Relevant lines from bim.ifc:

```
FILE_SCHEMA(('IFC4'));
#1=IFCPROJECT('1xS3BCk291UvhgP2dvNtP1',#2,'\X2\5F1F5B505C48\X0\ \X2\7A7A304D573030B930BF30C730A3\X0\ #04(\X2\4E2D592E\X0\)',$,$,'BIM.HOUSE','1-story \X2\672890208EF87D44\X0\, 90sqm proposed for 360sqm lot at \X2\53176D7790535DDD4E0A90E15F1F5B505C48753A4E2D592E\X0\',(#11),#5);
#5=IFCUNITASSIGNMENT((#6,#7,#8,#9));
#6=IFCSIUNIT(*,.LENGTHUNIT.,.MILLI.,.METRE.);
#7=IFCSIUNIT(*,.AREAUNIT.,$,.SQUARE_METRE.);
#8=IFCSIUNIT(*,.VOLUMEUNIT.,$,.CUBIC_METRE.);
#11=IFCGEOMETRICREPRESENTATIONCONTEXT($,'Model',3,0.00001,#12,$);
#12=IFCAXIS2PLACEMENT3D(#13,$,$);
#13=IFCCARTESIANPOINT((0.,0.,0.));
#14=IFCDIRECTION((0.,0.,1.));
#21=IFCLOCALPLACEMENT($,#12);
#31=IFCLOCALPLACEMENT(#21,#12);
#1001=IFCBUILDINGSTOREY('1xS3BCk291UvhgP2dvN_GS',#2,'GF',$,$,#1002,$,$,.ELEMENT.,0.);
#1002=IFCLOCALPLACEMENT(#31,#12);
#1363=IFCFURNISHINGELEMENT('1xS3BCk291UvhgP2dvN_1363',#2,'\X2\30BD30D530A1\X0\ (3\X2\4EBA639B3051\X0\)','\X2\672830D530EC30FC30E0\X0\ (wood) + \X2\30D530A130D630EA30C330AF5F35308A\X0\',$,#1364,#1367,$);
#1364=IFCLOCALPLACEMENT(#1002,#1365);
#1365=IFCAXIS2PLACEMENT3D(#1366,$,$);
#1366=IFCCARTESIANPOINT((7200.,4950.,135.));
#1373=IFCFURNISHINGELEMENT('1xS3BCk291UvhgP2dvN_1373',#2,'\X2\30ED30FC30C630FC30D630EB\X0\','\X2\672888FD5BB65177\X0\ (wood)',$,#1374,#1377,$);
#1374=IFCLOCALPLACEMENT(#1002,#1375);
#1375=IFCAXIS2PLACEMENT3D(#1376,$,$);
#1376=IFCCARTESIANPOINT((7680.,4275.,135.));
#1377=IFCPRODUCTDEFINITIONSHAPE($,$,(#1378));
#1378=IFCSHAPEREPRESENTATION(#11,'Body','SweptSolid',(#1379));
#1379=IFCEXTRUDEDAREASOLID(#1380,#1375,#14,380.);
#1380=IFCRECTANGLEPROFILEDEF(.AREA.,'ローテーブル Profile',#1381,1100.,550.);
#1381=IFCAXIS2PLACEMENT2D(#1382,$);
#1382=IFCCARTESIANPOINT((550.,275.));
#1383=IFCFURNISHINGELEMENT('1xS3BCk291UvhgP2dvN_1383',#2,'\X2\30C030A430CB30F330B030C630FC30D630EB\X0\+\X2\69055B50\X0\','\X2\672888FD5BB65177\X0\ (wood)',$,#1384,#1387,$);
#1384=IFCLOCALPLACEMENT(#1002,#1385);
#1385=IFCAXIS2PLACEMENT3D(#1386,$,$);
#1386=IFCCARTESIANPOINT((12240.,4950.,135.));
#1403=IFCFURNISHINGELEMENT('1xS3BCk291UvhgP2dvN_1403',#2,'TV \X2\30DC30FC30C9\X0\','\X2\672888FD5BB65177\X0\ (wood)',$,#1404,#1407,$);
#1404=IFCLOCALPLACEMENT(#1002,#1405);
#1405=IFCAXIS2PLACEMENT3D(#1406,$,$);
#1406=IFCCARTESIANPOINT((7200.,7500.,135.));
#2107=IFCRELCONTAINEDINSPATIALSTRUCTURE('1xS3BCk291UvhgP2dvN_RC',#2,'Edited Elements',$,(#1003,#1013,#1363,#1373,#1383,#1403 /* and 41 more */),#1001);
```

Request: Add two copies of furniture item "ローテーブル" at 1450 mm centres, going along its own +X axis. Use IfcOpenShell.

```python
import ifcopenshell
import ifcopenshell.api.geometry
import ifcopenshell.api.root
import ifcopenshell.util.element
import ifcopenshell.util.placement
import ifcopenshell.util.unit

model = ifcopenshell.open("bim.ifc")
unit_scale = ifcopenshell.util.unit.calculate_unit_scale(model)


def reuse_history(source, copy):
    """copy_class also copies each property set's owner history, people and application; keep the originals."""
    for rel in copy.IsDefinedBy:
        if rel.is_a("IfcRelDefinesByProperties") and (history := rel.RelatingPropertyDefinition.OwnerHistory):
            rel.RelatingPropertyDefinition.OwnerHistory = source.OwnerHistory
            ifcopenshell.util.element.remove_deep2(model, history)


source = model.by_id(1373)
base = ifcopenshell.util.placement.get_local_placement(source.ObjectPlacement)
step = base[:3, 0] * 1.45 / unit_scale

for i in range(1, 3):
    copy = ifcopenshell.api.root.copy_class(model, product=source)
    copy.Representation = ifcopenshell.util.element.copy_deep(
        model, source.Representation, exclude=["IfcGeometricRepresentationContext", "IfcRepresentationMap"]
    )
    reuse_history(source, copy)
    matrix = base.copy()
    matrix[:3, 3] += i * step
    print("added at", matrix[:3, 3].round(3) + 0.0)
    ifcopenshell.api.geometry.edit_object_placement(model, product=copy, matrix=matrix, is_si=False)

model.write("bim_edited.ifc")
```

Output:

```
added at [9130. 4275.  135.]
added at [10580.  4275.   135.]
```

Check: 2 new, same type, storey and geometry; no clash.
